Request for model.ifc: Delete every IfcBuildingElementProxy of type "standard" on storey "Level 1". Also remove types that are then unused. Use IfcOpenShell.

First a look at what the model holds.

```python
import ifcopenshell
import ifcopenshell.util.element

model = ifcopenshell.open("model.ifc")
print(model.schema)
storey = next(s for s in model.by_type("IfcBuildingStorey") if s.Name == "Level 1")
proxies = [e for e in ifcopenshell.util.element.get_decomposition(storey) if e.is_a("IfcBuildingElementProxy")]
seen = {}
for e in proxies:
    element_type = ifcopenshell.util.element.get_type(e)
    name = element_type.Name if element_type not in (None, e) else None
    seen[name] = seen.get(name, 0) + 1
for name, count in sorted(seen.items(), key=str):
    print(count, "x", name)
```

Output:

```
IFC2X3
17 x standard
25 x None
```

```python
import ifcopenshell
import ifcopenshell.api.root
import ifcopenshell.util.element

model = ifcopenshell.open("model.ifc")

storey = next(s for s in model.by_type("IfcBuildingStorey") if s.Name == "Level 1")
proxies = [e for e in ifcopenshell.util.element.get_decomposition(storey) if e.is_a("IfcBuildingElementProxy")]
targets = [e for e in proxies if (t := ifcopenshell.util.element.get_type(e)) not in (None, e) and t.Name == "standard"]
types = {ifcopenshell.util.element.get_type(e) for e in targets} - {None, *targets}

for e in targets:
    ifcopenshell.api.root.remove_product(model, product=e)
print(len(targets), "removed")

unused = [t for t in types if not ifcopenshell.util.element.get_types(t)]
for t in unused:
    ifcopenshell.api.root.remove_product(model, product=t)
print(len(unused), "unused types removed")

model.write("model-out.ifc")
```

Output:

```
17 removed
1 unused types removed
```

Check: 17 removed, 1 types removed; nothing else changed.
